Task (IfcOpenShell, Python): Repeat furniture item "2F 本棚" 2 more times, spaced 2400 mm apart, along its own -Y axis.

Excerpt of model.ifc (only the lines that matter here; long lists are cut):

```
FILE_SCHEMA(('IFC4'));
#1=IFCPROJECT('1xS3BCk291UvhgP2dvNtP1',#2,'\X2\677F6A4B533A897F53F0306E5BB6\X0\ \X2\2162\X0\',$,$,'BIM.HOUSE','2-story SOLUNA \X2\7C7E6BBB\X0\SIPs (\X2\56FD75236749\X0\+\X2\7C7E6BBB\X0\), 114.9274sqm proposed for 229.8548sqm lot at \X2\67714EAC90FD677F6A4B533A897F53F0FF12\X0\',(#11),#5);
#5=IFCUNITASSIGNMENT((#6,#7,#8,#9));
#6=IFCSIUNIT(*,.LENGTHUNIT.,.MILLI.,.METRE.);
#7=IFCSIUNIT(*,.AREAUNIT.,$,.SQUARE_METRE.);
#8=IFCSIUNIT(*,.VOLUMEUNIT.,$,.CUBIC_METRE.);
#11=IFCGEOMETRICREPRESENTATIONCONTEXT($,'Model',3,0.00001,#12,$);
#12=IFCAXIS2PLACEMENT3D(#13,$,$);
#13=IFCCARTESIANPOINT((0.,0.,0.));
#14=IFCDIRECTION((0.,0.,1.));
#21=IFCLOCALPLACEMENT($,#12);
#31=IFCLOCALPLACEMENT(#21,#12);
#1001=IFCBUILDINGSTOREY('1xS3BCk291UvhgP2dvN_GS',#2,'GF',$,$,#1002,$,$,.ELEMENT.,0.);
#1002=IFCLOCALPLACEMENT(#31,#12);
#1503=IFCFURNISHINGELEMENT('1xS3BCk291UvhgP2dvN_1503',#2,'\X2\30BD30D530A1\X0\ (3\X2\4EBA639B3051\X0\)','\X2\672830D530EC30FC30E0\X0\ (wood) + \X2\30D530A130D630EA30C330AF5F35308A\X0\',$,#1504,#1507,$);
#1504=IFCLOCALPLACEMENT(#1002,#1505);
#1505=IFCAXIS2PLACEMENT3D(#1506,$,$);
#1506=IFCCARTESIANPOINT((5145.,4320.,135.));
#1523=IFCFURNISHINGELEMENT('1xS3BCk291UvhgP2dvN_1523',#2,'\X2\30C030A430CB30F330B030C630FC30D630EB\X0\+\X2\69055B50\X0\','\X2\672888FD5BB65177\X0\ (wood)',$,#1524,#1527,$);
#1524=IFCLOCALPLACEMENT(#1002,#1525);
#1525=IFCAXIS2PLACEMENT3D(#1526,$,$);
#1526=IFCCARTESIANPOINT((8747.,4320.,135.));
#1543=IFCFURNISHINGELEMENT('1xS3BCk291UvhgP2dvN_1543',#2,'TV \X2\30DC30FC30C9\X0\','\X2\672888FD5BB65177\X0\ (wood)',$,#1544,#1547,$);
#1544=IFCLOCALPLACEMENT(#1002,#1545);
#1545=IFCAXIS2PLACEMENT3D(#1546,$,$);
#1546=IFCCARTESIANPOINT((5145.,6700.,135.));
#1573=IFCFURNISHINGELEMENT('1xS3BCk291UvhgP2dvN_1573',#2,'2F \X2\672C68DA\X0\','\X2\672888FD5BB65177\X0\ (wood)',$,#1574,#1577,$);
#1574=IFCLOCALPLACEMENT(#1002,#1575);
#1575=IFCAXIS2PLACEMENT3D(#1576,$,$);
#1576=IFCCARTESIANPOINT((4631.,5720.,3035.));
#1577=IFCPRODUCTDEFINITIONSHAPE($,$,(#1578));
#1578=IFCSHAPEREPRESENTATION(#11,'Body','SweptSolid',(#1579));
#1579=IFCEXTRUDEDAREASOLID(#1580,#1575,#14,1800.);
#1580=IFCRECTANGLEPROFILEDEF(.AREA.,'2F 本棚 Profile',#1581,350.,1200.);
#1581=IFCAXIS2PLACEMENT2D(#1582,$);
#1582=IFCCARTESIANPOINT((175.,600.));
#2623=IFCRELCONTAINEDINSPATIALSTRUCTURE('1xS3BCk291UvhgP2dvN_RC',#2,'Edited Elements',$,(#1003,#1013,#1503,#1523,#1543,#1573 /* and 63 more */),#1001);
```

```python
import ifcopenshell
import ifcopenshell.api.geometry
import ifcopenshell.api.root
import ifcopenshell.util.element
import ifcopenshell.util.placement

model = ifcopenshell.open("model.ifc")


def reuse_history(source, copy):
    """copy_class also copies each property set's owner history, people and application; keep the originals."""
    for rel in copy.IsDefinedBy:
        if rel.is_a("IfcRelDefinesByProperties") and (history := rel.RelatingPropertyDefinition.OwnerHistory):
            rel.RelatingPropertyDefinition.OwnerHistory = source.OwnerHistory
            ifcopenshell.util.element.remove_deep2(model, history)


source = model.by_guid("1xS3BCk291UvhgP2dvN_1573")
base = ifcopenshell.util.placement.get_local_placement(source.ObjectPlacement)
step = -base[:3, 1] * 2400.0

for i in range(1, 3):
    copy = ifcopenshell.api.root.copy_class(model, product=source)
    copy.Representation = ifcopenshell.util.element.copy_deep(
        model, source.Representation, exclude=["IfcGeometricRepresentationContext", "IfcRepresentationMap"]
    )
    reuse_history(source, copy)
    matrix = base.copy()
    matrix[:3, 3] += i * step
    print("added at", matrix[:3, 3].round(3) + 0.0)
    ifcopenshell.api.geometry.edit_object_placement(model, product=copy, matrix=matrix, is_si=False)

model.write("model_v2.ifc")
```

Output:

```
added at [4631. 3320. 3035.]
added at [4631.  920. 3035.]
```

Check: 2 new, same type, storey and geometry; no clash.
